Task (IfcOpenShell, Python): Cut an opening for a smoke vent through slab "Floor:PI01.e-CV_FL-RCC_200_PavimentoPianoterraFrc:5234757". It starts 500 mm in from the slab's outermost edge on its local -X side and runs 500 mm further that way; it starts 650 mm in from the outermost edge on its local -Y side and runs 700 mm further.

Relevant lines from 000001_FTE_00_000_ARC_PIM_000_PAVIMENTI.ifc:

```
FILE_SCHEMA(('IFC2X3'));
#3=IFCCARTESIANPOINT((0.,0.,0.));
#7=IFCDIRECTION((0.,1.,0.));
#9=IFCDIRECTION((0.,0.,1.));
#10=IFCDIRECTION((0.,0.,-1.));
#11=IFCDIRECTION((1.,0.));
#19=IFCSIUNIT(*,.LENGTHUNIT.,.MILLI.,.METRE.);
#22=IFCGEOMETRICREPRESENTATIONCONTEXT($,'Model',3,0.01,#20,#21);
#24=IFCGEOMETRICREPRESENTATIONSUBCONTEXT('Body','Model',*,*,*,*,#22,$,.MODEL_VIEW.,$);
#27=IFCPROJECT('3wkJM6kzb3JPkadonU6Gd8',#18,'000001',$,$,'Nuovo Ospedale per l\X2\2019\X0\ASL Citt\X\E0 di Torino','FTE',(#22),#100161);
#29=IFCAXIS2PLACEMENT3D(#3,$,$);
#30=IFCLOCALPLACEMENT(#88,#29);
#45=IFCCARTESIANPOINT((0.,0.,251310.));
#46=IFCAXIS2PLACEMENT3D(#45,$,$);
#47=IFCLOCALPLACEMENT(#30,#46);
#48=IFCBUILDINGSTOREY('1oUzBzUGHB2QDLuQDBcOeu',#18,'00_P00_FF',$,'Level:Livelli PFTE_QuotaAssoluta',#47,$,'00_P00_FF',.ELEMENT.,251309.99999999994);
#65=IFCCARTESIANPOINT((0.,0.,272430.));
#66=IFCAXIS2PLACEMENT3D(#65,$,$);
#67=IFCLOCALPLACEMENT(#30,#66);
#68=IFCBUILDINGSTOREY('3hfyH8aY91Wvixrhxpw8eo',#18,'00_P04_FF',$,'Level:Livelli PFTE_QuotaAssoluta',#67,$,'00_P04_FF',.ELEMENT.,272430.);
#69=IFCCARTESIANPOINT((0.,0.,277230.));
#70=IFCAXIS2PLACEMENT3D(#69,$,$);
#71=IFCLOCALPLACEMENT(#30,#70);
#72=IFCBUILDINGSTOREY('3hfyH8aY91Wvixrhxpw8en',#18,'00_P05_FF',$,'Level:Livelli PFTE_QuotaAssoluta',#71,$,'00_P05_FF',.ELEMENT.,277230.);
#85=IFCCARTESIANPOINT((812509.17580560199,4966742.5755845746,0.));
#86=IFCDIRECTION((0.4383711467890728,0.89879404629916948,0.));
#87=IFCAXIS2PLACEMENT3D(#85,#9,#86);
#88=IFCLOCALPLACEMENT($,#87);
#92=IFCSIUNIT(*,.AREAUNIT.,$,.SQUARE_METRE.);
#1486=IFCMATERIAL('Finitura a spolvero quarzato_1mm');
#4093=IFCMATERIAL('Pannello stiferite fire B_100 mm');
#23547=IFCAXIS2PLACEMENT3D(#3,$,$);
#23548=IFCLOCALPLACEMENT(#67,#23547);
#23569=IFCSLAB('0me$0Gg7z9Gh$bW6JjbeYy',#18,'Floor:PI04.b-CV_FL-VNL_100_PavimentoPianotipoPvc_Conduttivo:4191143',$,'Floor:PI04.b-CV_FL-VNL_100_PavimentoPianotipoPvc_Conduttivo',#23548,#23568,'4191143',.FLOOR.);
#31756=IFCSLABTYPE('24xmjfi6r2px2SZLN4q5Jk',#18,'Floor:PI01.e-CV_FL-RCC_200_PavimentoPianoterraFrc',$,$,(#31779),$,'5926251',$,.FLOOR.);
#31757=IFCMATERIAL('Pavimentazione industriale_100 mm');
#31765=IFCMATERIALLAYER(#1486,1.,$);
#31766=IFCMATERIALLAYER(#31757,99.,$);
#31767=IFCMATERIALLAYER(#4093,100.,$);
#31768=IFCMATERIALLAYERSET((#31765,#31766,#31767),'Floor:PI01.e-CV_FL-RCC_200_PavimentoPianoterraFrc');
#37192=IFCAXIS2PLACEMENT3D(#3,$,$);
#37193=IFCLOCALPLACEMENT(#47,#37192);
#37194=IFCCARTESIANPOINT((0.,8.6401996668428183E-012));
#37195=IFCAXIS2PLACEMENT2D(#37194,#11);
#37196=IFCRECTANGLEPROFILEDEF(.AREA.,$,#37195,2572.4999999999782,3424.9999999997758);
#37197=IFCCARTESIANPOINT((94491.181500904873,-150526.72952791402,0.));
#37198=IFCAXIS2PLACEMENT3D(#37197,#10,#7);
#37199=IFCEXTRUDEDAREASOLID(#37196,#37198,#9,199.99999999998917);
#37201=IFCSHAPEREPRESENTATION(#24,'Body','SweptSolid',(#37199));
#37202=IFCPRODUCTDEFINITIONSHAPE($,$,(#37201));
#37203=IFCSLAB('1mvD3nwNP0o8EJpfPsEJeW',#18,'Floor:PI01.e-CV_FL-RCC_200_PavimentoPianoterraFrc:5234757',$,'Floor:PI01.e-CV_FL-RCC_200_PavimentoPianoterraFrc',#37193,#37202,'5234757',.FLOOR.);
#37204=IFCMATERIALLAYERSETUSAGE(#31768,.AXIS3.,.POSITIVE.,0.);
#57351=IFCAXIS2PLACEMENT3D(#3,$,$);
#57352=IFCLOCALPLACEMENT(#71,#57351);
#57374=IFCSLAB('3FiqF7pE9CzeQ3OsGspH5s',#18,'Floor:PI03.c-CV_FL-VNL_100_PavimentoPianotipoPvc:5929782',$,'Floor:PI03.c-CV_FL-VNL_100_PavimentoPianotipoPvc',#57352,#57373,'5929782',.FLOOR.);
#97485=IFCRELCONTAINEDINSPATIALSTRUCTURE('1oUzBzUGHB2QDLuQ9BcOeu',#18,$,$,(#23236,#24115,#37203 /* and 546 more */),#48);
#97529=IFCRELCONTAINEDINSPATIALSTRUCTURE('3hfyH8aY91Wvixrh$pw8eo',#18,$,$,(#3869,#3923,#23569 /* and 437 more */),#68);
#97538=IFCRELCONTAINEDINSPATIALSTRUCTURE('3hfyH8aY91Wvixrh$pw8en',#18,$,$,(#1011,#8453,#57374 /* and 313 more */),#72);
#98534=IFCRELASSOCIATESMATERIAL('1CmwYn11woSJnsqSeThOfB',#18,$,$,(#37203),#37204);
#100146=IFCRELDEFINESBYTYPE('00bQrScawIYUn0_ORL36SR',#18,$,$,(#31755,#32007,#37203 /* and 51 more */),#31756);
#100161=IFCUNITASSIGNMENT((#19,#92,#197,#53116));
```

```python
import numpy as np
import ifcopenshell
import ifcopenshell.api.feature
import ifcopenshell.api.geometry
import ifcopenshell.api.root
import ifcopenshell.geom
import ifcopenshell.util.placement
import ifcopenshell.util.representation
import ifcopenshell.util.shape
import ifcopenshell.util.unit

model = ifcopenshell.open("000001_FTE_00_000_ARC_PIM_000_PAVIMENTI.ifc")
unit_scale = ifcopenshell.util.unit.calculate_unit_scale(model)
settings = ifcopenshell.geom.settings()


def volume(element):
    """Net volume in cubic metres, openings subtracted."""
    shape = ifcopenshell.geom.create_shape(settings, element)
    return ifcopenshell.util.shape.get_volume(shape.geometry)


slab = model.by_id(37203)
before = volume(slab)

# Extent in the slab's own axes, in metres. The edges named are its -X and -Y sides.
slab_shape = ifcopenshell.geom.create_shape(settings, slab)
vertices = ifcopenshell.util.shape.get_vertices(slab_shape.geometry)
x_min, y_min, bottom = vertices.min(axis=0)
top = vertices[:, 2].max()

opening = ifcopenshell.api.root.create_entity(model, ifc_class="IfcOpeningElement", name="Smoke vent opening")
context = ifcopenshell.util.representation.get_context(model, "Model", "Body", "MODEL_VIEW")
width, depth = 0.5, 0.7
outline = [(0.0, 0.0), (width, 0.0), (width, depth), (0.0, depth), (0.0, 0.0)]
# Overshoot both faces by 50 mm so the cut is clean.
shape = ifcopenshell.api.geometry.add_slab_representation(
    model, context=context, depth=top - bottom + 0.1, polyline=outline
)
ifcopenshell.api.geometry.assign_representation(model, product=opening, representation=shape)

matrix = ifcopenshell.util.placement.get_local_placement(slab.ObjectPlacement)
matrix[:, 3] = matrix @ np.append(np.array([x_min + 0.5, y_min + 0.65, bottom - 0.05]) / unit_scale, 1.0)
ifcopenshell.api.geometry.edit_object_placement(model, product=opening, matrix=matrix, is_si=False)
ifcopenshell.api.feature.add_feature(model, feature=opening, element=slab)

after = volume(slab)

print(f"slab volume {before:.3f} -> {after:.3f} m3")

model.write("000001_FTE_00_000_ARC_PIM_000_PAVIMENTI_v2.ifc")
```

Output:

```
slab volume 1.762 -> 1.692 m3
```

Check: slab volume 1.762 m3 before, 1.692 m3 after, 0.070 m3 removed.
